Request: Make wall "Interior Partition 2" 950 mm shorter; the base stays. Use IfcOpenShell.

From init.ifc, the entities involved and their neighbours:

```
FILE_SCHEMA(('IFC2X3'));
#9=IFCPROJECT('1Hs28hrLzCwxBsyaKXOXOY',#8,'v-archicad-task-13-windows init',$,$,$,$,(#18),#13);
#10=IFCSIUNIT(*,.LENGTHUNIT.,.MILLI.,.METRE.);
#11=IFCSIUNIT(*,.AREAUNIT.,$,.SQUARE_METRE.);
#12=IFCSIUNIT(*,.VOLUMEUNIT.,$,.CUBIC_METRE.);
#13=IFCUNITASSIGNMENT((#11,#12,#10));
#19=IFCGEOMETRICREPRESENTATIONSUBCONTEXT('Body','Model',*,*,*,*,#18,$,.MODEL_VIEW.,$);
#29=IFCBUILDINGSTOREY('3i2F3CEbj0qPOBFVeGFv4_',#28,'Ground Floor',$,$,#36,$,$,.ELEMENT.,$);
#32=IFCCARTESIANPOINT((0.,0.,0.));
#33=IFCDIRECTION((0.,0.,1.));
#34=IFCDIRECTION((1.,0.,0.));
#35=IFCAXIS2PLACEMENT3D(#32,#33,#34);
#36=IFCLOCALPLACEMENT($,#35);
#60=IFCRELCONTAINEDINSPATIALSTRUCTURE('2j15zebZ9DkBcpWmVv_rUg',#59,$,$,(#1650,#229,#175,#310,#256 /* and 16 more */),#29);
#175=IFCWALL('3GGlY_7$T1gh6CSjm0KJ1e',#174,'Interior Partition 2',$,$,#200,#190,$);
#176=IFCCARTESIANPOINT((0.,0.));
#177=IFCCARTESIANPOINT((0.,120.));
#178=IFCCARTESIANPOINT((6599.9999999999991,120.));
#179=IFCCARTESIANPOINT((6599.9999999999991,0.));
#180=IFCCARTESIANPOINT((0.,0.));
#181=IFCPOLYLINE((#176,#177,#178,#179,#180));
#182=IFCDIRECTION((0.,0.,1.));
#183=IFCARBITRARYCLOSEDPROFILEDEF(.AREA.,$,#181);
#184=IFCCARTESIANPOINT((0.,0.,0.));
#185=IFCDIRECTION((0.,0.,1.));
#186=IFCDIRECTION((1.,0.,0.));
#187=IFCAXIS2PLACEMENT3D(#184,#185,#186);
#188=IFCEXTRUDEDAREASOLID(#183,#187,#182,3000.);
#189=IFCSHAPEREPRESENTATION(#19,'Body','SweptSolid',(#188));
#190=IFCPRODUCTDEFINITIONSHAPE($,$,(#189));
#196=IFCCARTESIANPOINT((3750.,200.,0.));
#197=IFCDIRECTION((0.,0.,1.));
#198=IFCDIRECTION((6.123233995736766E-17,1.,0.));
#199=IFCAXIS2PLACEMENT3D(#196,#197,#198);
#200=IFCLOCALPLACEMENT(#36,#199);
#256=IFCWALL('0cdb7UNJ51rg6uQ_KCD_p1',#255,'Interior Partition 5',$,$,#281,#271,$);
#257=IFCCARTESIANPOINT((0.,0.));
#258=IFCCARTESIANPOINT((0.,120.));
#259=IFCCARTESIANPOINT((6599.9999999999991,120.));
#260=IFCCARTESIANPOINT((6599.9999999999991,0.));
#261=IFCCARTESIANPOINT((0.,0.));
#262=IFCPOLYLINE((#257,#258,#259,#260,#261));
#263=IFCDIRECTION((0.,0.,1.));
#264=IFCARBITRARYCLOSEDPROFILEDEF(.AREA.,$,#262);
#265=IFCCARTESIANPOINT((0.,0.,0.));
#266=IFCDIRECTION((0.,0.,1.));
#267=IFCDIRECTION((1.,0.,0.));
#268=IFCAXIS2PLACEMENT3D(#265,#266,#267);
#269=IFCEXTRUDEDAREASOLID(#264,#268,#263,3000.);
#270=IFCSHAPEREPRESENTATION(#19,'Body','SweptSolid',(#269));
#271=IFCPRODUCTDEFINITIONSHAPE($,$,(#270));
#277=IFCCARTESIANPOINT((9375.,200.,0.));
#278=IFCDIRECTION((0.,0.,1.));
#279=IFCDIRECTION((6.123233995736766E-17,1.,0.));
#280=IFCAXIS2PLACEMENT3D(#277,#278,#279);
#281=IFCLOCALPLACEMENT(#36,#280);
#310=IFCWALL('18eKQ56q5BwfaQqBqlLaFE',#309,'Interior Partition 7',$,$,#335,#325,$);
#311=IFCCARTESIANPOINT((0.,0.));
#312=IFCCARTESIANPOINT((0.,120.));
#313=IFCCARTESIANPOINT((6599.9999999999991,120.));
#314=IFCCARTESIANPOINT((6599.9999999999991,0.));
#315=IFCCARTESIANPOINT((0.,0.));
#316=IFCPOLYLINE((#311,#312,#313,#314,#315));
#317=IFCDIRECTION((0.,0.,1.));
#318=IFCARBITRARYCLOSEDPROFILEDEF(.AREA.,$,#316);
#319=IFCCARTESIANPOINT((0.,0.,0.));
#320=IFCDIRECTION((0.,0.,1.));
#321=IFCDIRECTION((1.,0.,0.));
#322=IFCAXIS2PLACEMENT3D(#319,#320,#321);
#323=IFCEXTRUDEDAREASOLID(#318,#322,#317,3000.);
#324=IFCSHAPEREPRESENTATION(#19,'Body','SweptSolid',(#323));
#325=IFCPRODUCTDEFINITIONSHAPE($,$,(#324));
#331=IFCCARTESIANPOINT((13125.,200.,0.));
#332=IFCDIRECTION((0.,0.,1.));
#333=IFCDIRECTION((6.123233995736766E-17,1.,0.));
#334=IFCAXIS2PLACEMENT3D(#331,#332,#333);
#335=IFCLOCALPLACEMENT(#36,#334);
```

```python
import ifcopenshell
import ifcopenshell.geom
import ifcopenshell.util.representation
import ifcopenshell.util.shape
import ifcopenshell.util.unit

model = ifcopenshell.open("init.ifc")
unit_scale = ifcopenshell.util.unit.calculate_unit_scale(model)
settings = ifcopenshell.geom.settings()


def volume(element):
    """Net volume in cubic metres, openings subtracted."""
    shape = ifcopenshell.geom.create_shape(settings, element)
    return ifcopenshell.util.shape.get_volume(shape.geometry)


wall = model.by_guid("3GGlY_7$T1gh6CSjm0KJ1e")
before = volume(wall)

body = ifcopenshell.util.representation.get_representation(wall, "Model", "Body")
solid = body.Items[0]
old_height = solid.Depth
solid.Depth -= 0.95 / unit_scale
after = volume(wall)

print(f"height {old_height:g} -> {solid.Depth:g}, volume {before:.3f} -> {after:.3f} m3")

model.write("init_rev.ifc")
```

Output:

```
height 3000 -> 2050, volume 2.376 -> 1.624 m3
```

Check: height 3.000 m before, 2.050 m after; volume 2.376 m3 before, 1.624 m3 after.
